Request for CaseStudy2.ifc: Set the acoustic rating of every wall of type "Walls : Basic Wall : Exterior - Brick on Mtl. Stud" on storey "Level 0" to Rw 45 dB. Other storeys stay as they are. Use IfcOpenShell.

First a look at what the model holds.

```python
import ifcopenshell
import ifcopenshell.util.element

model = ifcopenshell.open("CaseStudy2.ifc")
print(model.schema)
storey = next(s for s in model.by_type("IfcBuildingStorey") if s.Name == "Level 0")
walls = [e for e in ifcopenshell.util.element.get_decomposition(storey) if e.is_a("IfcWall")]
seen = {}
for e in walls:
    element_type = ifcopenshell.util.element.get_type(e)
    key = (element_type.Name if element_type != e and element_type else None, ifcopenshell.util.element.get_pset(e, "Pset_WallCommon", "AcousticRating"))
    seen[key] = seen.get(key, 0) + 1
for (name, value), count in sorted(seen.items(), key=str):
    print(count, "x", name, "|", value)
```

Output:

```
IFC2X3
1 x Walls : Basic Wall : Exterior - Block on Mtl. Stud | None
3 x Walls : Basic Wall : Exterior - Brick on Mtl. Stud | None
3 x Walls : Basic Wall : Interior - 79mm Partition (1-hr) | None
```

```python
import ifcopenshell
import ifcopenshell.api.pset
import ifcopenshell.util.element

model = ifcopenshell.open("CaseStudy2.ifc")

storey = next(s for s in model.by_type("IfcBuildingStorey") if s.Name == "Level 0")
walls = [e for e in ifcopenshell.util.element.get_decomposition(storey) if e.is_a("IfcWall")]

count = 0
for e in walls:
    element_type = ifcopenshell.util.element.get_type(e)
    if element_type in (None, e) or element_type.Name != "Walls : Basic Wall : Exterior - Brick on Mtl. Stud":
        continue
    # add_pset returns the element's existing set when there is one.
    pset = ifcopenshell.api.pset.add_pset(model, product=e, name="Pset_WallCommon")
    ifcopenshell.api.pset.edit_pset(model, pset=pset, properties={"AcousticRating": "Rw 45 dB"})
    count += 1

print(count, "walls updated")

model.write("CaseStudy2-out.ifc")
```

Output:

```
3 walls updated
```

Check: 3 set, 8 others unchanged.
